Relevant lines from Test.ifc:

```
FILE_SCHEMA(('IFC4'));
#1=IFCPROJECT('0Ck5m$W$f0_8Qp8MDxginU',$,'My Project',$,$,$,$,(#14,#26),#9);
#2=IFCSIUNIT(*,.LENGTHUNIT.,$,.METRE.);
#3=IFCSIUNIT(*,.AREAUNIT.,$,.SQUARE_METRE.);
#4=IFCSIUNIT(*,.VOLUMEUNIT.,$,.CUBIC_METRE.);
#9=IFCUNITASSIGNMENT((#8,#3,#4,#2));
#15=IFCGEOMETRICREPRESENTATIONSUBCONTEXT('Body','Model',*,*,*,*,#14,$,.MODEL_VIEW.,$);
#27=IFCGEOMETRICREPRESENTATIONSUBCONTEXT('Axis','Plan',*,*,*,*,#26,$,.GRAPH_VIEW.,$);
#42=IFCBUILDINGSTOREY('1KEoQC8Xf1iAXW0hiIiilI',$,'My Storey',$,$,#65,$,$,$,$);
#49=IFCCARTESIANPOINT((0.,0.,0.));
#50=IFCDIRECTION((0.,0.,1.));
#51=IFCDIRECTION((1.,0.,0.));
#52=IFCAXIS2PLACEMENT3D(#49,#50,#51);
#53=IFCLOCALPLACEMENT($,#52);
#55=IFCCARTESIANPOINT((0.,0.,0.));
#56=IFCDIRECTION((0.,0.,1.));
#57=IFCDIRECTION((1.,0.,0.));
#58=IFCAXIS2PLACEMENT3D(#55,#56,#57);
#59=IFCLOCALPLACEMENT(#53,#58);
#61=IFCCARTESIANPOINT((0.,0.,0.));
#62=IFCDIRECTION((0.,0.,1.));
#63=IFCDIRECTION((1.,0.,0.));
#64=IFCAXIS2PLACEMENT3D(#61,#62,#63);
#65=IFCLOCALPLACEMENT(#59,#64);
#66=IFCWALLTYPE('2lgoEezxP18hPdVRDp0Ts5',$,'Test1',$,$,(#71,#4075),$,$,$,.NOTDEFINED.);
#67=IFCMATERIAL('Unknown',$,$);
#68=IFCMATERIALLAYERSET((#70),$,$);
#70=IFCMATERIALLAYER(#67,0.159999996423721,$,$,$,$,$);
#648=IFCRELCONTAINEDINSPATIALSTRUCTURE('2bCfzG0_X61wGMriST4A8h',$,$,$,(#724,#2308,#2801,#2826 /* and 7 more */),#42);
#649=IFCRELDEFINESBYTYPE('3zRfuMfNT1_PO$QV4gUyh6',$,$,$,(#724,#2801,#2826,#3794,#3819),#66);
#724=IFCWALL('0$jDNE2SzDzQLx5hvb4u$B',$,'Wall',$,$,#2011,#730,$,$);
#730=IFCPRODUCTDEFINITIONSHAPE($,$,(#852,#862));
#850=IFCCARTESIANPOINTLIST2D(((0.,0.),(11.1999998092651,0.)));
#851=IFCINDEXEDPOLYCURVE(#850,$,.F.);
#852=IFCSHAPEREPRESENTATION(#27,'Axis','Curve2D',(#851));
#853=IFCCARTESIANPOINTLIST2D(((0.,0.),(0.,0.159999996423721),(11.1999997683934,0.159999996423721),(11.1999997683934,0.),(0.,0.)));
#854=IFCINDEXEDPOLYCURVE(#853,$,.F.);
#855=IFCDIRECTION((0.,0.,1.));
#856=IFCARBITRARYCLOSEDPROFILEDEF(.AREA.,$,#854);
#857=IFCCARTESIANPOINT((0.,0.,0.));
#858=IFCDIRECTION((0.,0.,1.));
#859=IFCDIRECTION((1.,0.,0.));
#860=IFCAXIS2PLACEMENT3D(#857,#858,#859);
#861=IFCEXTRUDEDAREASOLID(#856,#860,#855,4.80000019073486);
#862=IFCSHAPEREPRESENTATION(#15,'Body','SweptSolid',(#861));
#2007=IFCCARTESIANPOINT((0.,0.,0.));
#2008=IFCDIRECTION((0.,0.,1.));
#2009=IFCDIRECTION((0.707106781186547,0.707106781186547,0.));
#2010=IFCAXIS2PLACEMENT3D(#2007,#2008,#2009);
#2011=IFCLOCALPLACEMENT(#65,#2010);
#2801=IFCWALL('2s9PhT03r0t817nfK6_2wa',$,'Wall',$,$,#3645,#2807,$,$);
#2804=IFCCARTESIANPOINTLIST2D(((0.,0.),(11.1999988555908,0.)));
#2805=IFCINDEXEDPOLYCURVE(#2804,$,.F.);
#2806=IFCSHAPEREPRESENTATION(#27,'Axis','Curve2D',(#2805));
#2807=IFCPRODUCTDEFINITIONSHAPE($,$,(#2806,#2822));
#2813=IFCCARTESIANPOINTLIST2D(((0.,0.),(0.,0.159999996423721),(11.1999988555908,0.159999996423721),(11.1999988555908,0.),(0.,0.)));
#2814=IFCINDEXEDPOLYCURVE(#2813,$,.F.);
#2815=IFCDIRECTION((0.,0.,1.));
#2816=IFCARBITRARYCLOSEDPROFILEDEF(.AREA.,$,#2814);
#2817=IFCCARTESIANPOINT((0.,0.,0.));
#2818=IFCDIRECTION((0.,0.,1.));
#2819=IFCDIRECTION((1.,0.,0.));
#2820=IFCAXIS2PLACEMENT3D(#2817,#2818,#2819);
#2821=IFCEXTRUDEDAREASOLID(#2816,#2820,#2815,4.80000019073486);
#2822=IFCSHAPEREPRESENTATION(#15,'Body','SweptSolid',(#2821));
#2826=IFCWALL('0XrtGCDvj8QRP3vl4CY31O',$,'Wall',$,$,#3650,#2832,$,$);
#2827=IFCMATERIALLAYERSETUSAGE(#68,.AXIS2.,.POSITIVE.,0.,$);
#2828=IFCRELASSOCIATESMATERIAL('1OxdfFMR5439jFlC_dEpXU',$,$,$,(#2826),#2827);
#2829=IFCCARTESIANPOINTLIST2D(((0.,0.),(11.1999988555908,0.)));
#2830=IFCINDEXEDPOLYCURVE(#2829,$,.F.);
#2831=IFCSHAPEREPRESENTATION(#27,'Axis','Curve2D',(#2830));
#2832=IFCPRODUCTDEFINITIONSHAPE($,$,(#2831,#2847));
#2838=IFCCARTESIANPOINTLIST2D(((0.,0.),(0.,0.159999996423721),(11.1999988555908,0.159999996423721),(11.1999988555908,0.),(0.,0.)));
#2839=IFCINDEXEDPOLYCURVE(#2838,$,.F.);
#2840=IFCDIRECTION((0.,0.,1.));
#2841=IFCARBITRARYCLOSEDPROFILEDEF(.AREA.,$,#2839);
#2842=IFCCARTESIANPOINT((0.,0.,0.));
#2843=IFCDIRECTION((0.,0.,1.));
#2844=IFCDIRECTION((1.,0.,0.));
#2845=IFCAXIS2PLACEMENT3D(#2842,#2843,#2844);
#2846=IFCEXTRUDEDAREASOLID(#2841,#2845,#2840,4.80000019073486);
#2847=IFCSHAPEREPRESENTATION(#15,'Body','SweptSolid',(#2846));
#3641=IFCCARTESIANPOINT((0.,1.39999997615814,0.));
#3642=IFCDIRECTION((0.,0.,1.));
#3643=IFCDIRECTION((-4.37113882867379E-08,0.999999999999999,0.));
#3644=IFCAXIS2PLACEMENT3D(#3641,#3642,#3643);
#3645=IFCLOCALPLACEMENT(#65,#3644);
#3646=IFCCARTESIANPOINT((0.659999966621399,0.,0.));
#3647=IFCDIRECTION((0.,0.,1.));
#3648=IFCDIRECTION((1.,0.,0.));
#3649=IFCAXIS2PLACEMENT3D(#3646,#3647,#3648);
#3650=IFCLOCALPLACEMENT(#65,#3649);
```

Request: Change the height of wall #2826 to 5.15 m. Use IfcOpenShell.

```python
import ifcopenshell
import ifcopenshell.geom
import ifcopenshell.util.representation
import ifcopenshell.util.shape
import ifcopenshell.util.unit

model = ifcopenshell.open("Test.ifc")
unit_scale = ifcopenshell.util.unit.calculate_unit_scale(model)
settings = ifcopenshell.geom.settings()


def volume(element):
    """Net volume in cubic metres, openings subtracted."""
    shape = ifcopenshell.geom.create_shape(settings, element)
    return ifcopenshell.util.shape.get_volume(shape.geometry)


wall = model.by_guid("0XrtGCDvj8QRP3vl4CY31O")
before = volume(wall)

body = ifcopenshell.util.representation.get_representation(wall, "Model", "Body")
solid = body.Items[0]
old_height = solid.Depth
solid.Depth = 5.15 / unit_scale
after = volume(wall)

print(f"height {old_height:g} -> {solid.Depth:g}, volume {before:.3f} -> {after:.3f} m3")

model.write("Test_edited.ifc")
```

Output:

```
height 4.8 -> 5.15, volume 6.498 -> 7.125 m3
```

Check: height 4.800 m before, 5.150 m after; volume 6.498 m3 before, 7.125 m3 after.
